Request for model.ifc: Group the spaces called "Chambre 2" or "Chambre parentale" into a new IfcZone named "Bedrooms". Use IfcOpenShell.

First a look at what the model holds.

```python
import ifcopenshell

model = ifcopenshell.open("model.ifc")
print(model.schema)
seen = {}
for space in model.by_type("IfcSpace"):
    seen[space.LongName] = seen.get(space.LongName, 0) + 1
for name, count in sorted(seen.items(), key=str):
    print(count, "x", name)
print("zones:", [z.Name for z in model.by_type("IfcZone")][:20])
```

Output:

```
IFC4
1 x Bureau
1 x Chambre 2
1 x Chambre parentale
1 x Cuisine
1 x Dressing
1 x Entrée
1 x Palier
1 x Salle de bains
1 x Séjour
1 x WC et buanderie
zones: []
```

```python
import ifcopenshell
import ifcopenshell.api.group
import ifcopenshell.api.root

model = ifcopenshell.open("model.ifc")

names = {"Chambre 2", "Chambre parentale"}
spaces = [s for s in model.by_type("IfcSpace") if s.LongName in names]

zone = ifcopenshell.api.root.create_entity(model, ifc_class="IfcZone", name="Bedrooms")
ifcopenshell.api.group.assign_group(model, products=spaces, group=zone)
print(len(spaces), "spaces in", zone.Name)

model.write("model_edited.ifc")
```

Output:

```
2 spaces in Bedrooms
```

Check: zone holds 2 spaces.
